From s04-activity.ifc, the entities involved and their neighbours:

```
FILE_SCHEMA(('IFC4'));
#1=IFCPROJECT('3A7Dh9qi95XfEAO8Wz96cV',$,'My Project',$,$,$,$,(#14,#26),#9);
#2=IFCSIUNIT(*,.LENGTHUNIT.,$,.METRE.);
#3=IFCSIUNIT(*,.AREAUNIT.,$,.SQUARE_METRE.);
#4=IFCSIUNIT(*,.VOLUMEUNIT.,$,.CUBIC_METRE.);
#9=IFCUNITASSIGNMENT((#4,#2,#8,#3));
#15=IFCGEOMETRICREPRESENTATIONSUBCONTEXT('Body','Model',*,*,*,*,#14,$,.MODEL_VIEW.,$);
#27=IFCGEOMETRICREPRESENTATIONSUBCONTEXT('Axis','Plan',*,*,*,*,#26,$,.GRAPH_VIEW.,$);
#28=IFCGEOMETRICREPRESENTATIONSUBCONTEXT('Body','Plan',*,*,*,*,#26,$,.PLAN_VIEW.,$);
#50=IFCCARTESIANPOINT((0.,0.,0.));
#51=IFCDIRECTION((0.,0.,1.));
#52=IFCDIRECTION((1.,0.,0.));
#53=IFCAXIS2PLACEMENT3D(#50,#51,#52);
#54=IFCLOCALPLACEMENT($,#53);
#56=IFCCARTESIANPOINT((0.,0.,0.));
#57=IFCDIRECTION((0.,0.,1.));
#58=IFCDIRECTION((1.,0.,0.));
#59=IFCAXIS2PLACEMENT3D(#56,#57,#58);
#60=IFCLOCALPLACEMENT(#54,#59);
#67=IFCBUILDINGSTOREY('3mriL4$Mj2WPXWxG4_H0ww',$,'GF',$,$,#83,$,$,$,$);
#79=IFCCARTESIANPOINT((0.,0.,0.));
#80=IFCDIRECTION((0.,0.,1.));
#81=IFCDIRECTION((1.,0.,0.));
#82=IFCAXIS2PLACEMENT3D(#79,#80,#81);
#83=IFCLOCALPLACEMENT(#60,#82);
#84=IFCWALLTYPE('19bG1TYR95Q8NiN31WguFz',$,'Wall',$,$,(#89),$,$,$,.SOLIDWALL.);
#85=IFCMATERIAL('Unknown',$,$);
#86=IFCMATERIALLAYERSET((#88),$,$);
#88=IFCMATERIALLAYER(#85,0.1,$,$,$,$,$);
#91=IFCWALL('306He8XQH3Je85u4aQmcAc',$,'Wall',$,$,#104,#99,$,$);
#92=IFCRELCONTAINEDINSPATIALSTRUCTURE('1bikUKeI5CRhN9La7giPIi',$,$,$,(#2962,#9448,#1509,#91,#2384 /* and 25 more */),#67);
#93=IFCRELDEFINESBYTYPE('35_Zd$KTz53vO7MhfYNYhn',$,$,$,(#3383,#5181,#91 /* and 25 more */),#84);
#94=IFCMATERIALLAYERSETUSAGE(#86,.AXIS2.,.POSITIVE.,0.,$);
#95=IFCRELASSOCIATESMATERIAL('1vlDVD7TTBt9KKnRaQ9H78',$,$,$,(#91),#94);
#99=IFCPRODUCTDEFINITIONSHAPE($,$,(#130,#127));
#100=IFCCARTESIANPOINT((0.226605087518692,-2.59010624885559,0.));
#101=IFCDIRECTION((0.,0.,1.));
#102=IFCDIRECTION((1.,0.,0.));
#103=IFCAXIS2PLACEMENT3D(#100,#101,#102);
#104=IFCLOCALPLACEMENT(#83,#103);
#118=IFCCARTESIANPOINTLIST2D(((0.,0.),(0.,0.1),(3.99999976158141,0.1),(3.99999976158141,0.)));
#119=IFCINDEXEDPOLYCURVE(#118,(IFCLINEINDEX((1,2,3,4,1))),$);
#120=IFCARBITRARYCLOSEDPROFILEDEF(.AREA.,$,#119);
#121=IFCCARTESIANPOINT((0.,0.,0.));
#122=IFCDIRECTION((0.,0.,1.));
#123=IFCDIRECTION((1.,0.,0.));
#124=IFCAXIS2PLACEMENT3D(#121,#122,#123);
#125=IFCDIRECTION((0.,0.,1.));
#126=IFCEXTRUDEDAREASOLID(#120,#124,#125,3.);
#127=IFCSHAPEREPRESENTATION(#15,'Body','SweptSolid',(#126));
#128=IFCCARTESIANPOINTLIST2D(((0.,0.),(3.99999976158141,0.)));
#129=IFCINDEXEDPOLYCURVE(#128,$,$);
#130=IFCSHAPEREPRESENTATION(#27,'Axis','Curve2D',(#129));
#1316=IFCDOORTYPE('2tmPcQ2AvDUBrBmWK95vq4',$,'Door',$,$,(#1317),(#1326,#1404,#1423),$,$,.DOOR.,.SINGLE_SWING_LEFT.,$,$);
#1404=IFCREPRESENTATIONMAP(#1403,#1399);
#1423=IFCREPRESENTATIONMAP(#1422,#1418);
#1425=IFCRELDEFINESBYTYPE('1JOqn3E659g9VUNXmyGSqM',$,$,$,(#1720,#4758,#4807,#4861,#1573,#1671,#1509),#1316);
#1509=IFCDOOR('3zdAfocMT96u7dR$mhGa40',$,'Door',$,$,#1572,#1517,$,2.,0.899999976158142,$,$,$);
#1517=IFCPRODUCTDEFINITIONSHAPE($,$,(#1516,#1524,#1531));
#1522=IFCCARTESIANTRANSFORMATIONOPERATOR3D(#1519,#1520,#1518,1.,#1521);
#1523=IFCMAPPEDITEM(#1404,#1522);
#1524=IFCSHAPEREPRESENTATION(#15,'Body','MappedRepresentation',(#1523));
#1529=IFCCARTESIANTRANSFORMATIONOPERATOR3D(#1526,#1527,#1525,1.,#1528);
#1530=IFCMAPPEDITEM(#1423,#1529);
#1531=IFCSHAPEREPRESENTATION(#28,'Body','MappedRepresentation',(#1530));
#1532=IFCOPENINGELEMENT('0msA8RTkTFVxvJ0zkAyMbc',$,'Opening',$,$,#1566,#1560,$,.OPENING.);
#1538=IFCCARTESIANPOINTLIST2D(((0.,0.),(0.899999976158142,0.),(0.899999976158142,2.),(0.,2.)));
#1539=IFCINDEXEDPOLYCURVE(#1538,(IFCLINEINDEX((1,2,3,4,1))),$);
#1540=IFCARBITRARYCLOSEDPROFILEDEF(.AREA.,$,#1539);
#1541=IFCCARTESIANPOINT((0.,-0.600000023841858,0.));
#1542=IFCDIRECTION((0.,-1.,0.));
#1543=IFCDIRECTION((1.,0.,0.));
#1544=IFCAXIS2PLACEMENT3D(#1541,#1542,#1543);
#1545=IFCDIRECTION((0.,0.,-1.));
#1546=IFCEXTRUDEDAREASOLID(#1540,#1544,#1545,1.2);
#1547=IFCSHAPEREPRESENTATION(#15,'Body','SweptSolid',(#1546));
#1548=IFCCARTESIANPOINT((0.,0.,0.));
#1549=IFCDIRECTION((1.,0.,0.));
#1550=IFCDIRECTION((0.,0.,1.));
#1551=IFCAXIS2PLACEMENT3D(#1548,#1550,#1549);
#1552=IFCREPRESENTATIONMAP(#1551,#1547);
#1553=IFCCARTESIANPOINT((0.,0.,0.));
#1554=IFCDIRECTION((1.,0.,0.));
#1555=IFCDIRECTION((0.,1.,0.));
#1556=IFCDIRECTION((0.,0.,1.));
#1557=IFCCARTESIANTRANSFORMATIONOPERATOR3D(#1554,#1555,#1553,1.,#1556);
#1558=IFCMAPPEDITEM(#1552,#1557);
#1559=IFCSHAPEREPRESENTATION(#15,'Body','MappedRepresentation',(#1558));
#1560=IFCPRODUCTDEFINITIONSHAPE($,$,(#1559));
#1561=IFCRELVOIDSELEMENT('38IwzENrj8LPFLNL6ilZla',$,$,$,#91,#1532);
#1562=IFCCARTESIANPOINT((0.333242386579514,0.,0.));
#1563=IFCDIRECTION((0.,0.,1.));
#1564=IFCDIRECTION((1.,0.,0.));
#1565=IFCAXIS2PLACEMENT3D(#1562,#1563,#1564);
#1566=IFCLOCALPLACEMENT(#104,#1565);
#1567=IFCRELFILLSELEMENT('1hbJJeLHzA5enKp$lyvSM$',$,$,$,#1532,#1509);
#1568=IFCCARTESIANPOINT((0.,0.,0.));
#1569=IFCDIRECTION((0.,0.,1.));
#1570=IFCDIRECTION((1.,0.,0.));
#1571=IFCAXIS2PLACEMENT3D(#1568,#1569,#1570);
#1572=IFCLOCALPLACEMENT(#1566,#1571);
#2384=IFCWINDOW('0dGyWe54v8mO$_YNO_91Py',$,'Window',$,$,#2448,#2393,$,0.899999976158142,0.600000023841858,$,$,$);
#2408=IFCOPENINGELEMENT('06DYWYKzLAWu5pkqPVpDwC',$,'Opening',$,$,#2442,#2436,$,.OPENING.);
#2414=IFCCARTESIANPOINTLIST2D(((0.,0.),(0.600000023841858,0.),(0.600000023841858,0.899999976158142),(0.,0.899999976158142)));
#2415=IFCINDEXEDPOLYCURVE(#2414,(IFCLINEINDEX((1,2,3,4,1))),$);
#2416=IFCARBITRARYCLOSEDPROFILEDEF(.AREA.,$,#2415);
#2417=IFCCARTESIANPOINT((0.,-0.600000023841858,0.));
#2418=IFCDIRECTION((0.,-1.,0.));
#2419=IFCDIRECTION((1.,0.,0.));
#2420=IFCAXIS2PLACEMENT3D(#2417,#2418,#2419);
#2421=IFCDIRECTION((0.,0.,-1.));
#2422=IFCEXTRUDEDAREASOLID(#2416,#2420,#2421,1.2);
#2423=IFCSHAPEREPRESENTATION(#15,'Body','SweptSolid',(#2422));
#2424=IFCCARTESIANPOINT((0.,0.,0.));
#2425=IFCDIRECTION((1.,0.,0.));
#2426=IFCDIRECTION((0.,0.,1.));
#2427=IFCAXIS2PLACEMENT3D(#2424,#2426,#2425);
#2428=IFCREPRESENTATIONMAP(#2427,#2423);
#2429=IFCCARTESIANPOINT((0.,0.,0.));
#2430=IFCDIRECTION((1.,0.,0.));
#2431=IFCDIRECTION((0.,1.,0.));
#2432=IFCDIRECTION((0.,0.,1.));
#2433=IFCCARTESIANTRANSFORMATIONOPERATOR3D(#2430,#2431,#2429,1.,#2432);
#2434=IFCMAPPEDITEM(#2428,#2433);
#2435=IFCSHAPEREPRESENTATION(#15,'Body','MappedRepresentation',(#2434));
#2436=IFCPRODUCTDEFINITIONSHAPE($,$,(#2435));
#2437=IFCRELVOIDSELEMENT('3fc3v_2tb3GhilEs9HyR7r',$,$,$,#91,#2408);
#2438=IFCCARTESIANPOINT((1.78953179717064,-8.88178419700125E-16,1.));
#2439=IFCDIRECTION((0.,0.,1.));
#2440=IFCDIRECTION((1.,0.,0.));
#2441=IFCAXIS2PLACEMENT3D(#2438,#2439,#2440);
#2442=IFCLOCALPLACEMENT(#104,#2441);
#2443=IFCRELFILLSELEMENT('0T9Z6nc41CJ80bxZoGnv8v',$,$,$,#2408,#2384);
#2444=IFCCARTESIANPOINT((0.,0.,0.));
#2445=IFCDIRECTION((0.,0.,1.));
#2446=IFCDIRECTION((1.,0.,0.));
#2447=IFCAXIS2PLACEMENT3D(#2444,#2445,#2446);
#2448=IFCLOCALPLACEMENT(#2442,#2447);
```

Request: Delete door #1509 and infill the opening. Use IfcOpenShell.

```python
import ifcopenshell
import ifcopenshell.api.feature
import ifcopenshell.api.root
import ifcopenshell.geom
import ifcopenshell.util.shape

model = ifcopenshell.open("s04-activity.ifc")
settings = ifcopenshell.geom.settings()


def volume(element):
    """Net volume in cubic metres, openings subtracted."""
    shape = ifcopenshell.geom.create_shape(settings, element)
    return ifcopenshell.util.shape.get_volume(shape.geometry)


door = model.by_guid("3zdAfocMT96u7dR$mhGa40")
opening = door.FillsVoids[0].RelatingOpeningElement
wall = opening.VoidsElements[0].RelatingBuildingElement
before = volume(wall)

ifcopenshell.api.root.remove_product(model, product=door)
ifcopenshell.api.feature.remove_feature(model, feature=opening)

after = volume(wall)

print(f"wall volume {before:.3f} -> {after:.3f} m3")

model.write("s04-activity_v2.ifc")
```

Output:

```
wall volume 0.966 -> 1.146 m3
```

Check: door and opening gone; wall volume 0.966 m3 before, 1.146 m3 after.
